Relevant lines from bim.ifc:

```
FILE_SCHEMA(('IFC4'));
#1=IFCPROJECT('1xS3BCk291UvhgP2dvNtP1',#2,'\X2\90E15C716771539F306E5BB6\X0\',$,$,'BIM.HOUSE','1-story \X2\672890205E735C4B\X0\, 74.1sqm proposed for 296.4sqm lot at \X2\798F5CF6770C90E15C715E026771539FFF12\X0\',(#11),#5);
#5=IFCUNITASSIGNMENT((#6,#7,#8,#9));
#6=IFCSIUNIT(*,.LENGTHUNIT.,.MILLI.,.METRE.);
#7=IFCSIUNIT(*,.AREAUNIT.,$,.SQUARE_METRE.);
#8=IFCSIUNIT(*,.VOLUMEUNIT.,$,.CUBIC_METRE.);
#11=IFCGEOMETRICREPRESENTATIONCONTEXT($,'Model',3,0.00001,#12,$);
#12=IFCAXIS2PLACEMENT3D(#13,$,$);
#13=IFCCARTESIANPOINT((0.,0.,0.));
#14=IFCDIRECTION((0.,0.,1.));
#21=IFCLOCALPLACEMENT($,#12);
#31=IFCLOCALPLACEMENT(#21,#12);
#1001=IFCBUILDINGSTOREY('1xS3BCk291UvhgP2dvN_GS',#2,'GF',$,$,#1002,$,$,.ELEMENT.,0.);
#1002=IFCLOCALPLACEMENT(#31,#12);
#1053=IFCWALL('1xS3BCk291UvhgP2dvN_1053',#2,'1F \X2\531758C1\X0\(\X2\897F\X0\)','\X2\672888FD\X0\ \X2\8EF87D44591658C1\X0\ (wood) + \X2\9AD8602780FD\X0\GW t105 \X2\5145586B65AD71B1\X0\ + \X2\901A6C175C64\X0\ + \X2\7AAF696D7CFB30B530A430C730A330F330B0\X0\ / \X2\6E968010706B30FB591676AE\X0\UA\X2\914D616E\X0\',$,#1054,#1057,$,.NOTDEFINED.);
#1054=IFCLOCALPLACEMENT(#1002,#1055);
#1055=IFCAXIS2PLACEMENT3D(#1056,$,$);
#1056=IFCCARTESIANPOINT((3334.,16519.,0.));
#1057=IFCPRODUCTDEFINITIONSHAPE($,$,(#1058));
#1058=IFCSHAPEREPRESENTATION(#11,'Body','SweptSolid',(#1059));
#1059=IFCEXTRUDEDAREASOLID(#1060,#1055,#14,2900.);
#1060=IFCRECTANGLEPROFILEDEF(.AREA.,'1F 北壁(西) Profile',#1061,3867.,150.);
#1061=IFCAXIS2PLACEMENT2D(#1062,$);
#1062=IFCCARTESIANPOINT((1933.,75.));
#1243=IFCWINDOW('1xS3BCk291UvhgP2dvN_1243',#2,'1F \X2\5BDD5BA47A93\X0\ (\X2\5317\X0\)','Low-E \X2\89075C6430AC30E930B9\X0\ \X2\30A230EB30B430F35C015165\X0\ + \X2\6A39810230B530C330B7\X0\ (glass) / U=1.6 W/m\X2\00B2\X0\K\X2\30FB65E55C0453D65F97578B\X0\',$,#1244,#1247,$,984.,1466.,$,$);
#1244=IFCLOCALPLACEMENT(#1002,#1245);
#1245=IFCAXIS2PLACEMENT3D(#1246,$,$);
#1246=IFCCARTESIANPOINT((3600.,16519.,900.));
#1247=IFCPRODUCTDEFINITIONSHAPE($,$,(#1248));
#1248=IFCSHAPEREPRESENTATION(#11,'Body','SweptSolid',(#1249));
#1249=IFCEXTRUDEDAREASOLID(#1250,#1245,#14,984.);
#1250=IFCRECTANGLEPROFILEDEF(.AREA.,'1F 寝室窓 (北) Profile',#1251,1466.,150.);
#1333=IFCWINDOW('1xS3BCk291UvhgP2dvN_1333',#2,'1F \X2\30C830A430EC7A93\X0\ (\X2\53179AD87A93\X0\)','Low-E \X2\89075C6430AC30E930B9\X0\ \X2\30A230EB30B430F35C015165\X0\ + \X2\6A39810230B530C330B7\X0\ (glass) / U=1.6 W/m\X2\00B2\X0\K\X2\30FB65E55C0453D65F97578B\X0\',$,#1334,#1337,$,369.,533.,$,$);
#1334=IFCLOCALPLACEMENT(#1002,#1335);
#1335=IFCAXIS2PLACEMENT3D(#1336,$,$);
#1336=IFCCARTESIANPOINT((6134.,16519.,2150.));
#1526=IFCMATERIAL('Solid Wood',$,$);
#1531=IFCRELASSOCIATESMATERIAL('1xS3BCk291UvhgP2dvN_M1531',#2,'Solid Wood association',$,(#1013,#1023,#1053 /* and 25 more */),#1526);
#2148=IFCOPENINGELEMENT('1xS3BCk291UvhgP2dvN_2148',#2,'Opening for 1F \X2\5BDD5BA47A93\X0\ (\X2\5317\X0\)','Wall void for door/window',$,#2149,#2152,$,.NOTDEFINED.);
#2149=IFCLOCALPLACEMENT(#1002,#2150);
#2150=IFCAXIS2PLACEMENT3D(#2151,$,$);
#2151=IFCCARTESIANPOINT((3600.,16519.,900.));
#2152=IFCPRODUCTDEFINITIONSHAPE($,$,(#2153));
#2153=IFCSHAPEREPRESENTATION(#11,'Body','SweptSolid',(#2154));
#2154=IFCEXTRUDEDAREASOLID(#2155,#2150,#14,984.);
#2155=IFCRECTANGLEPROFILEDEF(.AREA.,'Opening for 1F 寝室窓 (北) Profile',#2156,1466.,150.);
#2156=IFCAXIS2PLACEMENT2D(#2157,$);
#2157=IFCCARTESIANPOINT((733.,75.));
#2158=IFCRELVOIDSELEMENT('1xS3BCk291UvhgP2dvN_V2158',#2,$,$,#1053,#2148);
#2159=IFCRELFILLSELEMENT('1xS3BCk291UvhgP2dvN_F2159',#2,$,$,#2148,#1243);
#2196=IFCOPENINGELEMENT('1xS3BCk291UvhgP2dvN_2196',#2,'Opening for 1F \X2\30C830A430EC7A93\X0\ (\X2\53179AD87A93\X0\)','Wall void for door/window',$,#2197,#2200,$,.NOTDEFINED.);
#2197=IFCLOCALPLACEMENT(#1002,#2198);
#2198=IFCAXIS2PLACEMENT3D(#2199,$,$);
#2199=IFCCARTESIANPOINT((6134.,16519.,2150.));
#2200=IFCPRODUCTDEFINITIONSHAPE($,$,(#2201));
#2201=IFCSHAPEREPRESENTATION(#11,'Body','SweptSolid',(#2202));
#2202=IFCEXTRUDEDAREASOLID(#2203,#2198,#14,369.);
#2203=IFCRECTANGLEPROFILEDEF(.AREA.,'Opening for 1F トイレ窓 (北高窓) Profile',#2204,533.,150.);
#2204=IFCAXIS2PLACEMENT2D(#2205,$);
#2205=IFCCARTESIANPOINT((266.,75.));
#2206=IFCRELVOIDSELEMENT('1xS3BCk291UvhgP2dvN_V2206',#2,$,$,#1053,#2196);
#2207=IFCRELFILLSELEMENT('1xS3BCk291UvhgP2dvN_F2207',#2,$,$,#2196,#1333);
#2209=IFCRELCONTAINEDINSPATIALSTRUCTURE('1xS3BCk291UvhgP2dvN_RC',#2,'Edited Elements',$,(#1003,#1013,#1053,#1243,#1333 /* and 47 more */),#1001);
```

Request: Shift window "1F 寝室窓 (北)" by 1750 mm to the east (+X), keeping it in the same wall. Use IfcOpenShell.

```python
import ifcopenshell
import ifcopenshell.api.geometry
import ifcopenshell.util.placement
import ifcopenshell.util.unit

model = ifcopenshell.open("bim.ifc")
unit_scale = ifcopenshell.util.unit.calculate_unit_scale(model)

window = model.by_guid("1xS3BCk291UvhgP2dvN_1243")
opening = window.FillsVoids[0].RelatingOpeningElement
wall = opening.VoidsElements[0].RelatingBuildingElement

wall_matrix = ifcopenshell.util.placement.get_local_placement(wall.ObjectPlacement)
shift = wall_matrix[:3, 0] * 1.75 / unit_scale
before = ifcopenshell.util.placement.get_local_placement(window.ObjectPlacement)[:3, 3].copy()

# The window is not placed relative to its opening, so move both.
for product in (opening, window):
    matrix = ifcopenshell.util.placement.get_local_placement(product.ObjectPlacement)
    matrix[:3, 3] += shift
    ifcopenshell.api.geometry.edit_object_placement(model, product=product, matrix=matrix, is_si=False)

after = ifcopenshell.util.placement.get_local_placement(window.ObjectPlacement)[:3, 3]
print("window moved by", (after - before).round(3) + 0.0)

model.write("bim_rev.ifc")
```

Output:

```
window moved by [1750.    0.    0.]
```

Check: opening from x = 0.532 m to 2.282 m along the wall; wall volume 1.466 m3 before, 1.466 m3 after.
